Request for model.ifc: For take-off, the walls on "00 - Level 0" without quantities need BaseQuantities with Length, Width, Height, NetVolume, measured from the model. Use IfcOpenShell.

First a look at what the model holds.

```python
import ifcopenshell
import ifcopenshell.util.element
import ifcopenshell.util.unit

model = ifcopenshell.open("model.ifc")
print(model.schema)
for unit_type in ("LENGTHUNIT", "AREAUNIT", "VOLUMEUNIT"):
    print(unit_type, ifcopenshell.util.unit.calculate_unit_scale(model, unit_type))
storey = next(s for s in model.by_type("IfcBuildingStorey") if s.Name == "00 - Level 0")
walls = [e for e in ifcopenshell.util.element.get_decomposition(storey) if e.is_a("IfcWall")]
for e in sorted(walls, key=lambda e: e.id()):
    print(e.id(), e.is_a(), e.Name, list(ifcopenshell.util.element.get_psets(e, qtos_only=True)), sep=" | ")
```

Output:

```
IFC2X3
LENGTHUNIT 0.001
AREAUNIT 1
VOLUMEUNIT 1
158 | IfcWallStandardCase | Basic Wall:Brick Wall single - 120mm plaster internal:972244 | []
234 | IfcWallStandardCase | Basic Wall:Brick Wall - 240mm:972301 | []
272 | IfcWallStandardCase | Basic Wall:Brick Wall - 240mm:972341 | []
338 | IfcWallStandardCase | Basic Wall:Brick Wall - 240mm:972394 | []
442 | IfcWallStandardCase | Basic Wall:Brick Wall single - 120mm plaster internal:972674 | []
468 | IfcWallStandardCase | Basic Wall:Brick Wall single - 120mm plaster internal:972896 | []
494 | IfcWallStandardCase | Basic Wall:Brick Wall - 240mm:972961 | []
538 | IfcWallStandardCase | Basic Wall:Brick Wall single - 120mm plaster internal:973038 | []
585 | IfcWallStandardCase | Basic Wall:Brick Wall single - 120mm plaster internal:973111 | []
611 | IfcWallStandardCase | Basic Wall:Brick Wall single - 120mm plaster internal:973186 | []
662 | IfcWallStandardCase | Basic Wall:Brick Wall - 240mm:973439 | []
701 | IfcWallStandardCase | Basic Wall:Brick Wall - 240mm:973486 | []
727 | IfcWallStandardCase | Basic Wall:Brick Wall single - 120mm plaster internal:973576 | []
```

```python
import ifcopenshell
import ifcopenshell.api.pset
import ifcopenshell.geom
import ifcopenshell.util.element
import ifcopenshell.util.shape
import ifcopenshell.util.unit

model = ifcopenshell.open("model.ifc")
unit_scale = ifcopenshell.util.unit.calculate_unit_scale(model)
volume_scale = ifcopenshell.util.unit.calculate_unit_scale(model, "VOLUMEUNIT")
settings = ifcopenshell.geom.settings()

storey = next(s for s in model.by_type("IfcBuildingStorey") if s.Name == "00 - Level 0")
walls = [e for e in ifcopenshell.util.element.get_decomposition(storey) if e.is_a("IfcWall")]

for e in sorted(walls, key=lambda e: e.id()):
    if ifcopenshell.util.element.get_psets(e, qtos_only=True, should_inherit=False):
        continue
    # Geometry comes back in metres, in the element's own axes.
    shape = ifcopenshell.geom.create_shape(settings, e)
    values = {
        "Length": ifcopenshell.util.shape.get_x(shape.geometry) / unit_scale,
        "Width": ifcopenshell.util.shape.get_y(shape.geometry) / unit_scale,
        "Height": ifcopenshell.util.shape.get_z(shape.geometry) / unit_scale,
        "NetVolume": ifcopenshell.util.shape.get_volume(shape.geometry) / volume_scale,
    }
    qto = ifcopenshell.api.pset.add_qto(model, product=e, name="BaseQuantities")
    ifcopenshell.api.pset.edit_qto(model, qto=qto, properties=values)
    print(e.id(), {k: round(v, 3) for k, v in values.items()})

model.write("model-out.ifc")
```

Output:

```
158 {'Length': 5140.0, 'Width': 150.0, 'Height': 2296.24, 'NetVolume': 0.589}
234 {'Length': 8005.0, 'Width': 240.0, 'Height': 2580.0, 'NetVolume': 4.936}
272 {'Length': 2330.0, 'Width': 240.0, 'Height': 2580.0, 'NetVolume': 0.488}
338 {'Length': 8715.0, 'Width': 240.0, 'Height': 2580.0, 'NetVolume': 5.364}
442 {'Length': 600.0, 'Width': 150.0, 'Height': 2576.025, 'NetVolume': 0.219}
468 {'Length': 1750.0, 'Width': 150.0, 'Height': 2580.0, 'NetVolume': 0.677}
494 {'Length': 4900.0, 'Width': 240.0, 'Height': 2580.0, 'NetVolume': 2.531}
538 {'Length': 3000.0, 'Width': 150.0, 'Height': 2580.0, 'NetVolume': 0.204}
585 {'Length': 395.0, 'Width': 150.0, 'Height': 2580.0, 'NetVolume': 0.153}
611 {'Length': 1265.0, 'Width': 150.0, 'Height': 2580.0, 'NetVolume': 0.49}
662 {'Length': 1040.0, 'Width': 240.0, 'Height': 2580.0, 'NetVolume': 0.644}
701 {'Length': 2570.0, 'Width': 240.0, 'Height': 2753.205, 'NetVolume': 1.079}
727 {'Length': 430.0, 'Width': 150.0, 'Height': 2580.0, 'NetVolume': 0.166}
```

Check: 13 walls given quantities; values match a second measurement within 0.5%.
